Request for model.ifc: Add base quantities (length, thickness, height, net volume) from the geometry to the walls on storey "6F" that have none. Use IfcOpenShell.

First a look at what the model holds.

```python
import ifcopenshell
import ifcopenshell.util.element
import ifcopenshell.util.unit

model = ifcopenshell.open("model.ifc")
print(model.schema)
for unit_type in ("LENGTHUNIT", "AREAUNIT", "VOLUMEUNIT"):
    print(unit_type, ifcopenshell.util.unit.calculate_unit_scale(model, unit_type))
storey = next(s for s in model.by_type("IfcBuildingStorey") if s.Name == "6F")
walls = [e for e in ifcopenshell.util.element.get_decomposition(storey) if e.is_a("IfcWall")]
for e in sorted(walls, key=lambda e: e.id()):
    print(e.id(), e.is_a(), e.Name, list(ifcopenshell.util.element.get_psets(e, qtos_only=True)), sep=" | ")
```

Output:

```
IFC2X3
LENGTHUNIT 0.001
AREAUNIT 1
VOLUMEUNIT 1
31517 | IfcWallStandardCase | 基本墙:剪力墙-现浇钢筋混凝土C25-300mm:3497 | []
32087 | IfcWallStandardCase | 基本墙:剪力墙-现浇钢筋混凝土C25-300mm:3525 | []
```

```python
import ifcopenshell
import ifcopenshell.api.pset
import ifcopenshell.geom
import ifcopenshell.util.element
import ifcopenshell.util.shape
import ifcopenshell.util.unit

model = ifcopenshell.open("model.ifc")
unit_scale = ifcopenshell.util.unit.calculate_unit_scale(model)
volume_scale = ifcopenshell.util.unit.calculate_unit_scale(model, "VOLUMEUNIT")
settings = ifcopenshell.geom.settings()

storey = next(s for s in model.by_type("IfcBuildingStorey") if s.Name == "6F")
walls = [e for e in ifcopenshell.util.element.get_decomposition(storey) if e.is_a("IfcWall")]

for e in sorted(walls, key=lambda e: e.id()):
    if ifcopenshell.util.element.get_psets(e, qtos_only=True, should_inherit=False):
        continue
    # Geometry comes back in metres, in the element's own axes.
    shape = ifcopenshell.geom.create_shape(settings, e)
    values = {
        "Length": ifcopenshell.util.shape.get_x(shape.geometry) / unit_scale,
        "Width": ifcopenshell.util.shape.get_y(shape.geometry) / unit_scale,
        "Height": ifcopenshell.util.shape.get_z(shape.geometry) / unit_scale,
        "NetVolume": ifcopenshell.util.shape.get_volume(shape.geometry) / volume_scale,
    }
    qto = ifcopenshell.api.pset.add_qto(model, product=e, name="BaseQuantities")
    ifcopenshell.api.pset.edit_qto(model, qto=qto, properties=values)
    print(e.id(), {k: round(v, 3) for k, v in values.items()})

model.write("model_v2.ifc")
```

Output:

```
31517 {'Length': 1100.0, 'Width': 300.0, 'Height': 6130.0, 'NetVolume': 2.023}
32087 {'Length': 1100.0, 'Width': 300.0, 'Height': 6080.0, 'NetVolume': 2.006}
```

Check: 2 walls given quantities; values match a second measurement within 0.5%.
